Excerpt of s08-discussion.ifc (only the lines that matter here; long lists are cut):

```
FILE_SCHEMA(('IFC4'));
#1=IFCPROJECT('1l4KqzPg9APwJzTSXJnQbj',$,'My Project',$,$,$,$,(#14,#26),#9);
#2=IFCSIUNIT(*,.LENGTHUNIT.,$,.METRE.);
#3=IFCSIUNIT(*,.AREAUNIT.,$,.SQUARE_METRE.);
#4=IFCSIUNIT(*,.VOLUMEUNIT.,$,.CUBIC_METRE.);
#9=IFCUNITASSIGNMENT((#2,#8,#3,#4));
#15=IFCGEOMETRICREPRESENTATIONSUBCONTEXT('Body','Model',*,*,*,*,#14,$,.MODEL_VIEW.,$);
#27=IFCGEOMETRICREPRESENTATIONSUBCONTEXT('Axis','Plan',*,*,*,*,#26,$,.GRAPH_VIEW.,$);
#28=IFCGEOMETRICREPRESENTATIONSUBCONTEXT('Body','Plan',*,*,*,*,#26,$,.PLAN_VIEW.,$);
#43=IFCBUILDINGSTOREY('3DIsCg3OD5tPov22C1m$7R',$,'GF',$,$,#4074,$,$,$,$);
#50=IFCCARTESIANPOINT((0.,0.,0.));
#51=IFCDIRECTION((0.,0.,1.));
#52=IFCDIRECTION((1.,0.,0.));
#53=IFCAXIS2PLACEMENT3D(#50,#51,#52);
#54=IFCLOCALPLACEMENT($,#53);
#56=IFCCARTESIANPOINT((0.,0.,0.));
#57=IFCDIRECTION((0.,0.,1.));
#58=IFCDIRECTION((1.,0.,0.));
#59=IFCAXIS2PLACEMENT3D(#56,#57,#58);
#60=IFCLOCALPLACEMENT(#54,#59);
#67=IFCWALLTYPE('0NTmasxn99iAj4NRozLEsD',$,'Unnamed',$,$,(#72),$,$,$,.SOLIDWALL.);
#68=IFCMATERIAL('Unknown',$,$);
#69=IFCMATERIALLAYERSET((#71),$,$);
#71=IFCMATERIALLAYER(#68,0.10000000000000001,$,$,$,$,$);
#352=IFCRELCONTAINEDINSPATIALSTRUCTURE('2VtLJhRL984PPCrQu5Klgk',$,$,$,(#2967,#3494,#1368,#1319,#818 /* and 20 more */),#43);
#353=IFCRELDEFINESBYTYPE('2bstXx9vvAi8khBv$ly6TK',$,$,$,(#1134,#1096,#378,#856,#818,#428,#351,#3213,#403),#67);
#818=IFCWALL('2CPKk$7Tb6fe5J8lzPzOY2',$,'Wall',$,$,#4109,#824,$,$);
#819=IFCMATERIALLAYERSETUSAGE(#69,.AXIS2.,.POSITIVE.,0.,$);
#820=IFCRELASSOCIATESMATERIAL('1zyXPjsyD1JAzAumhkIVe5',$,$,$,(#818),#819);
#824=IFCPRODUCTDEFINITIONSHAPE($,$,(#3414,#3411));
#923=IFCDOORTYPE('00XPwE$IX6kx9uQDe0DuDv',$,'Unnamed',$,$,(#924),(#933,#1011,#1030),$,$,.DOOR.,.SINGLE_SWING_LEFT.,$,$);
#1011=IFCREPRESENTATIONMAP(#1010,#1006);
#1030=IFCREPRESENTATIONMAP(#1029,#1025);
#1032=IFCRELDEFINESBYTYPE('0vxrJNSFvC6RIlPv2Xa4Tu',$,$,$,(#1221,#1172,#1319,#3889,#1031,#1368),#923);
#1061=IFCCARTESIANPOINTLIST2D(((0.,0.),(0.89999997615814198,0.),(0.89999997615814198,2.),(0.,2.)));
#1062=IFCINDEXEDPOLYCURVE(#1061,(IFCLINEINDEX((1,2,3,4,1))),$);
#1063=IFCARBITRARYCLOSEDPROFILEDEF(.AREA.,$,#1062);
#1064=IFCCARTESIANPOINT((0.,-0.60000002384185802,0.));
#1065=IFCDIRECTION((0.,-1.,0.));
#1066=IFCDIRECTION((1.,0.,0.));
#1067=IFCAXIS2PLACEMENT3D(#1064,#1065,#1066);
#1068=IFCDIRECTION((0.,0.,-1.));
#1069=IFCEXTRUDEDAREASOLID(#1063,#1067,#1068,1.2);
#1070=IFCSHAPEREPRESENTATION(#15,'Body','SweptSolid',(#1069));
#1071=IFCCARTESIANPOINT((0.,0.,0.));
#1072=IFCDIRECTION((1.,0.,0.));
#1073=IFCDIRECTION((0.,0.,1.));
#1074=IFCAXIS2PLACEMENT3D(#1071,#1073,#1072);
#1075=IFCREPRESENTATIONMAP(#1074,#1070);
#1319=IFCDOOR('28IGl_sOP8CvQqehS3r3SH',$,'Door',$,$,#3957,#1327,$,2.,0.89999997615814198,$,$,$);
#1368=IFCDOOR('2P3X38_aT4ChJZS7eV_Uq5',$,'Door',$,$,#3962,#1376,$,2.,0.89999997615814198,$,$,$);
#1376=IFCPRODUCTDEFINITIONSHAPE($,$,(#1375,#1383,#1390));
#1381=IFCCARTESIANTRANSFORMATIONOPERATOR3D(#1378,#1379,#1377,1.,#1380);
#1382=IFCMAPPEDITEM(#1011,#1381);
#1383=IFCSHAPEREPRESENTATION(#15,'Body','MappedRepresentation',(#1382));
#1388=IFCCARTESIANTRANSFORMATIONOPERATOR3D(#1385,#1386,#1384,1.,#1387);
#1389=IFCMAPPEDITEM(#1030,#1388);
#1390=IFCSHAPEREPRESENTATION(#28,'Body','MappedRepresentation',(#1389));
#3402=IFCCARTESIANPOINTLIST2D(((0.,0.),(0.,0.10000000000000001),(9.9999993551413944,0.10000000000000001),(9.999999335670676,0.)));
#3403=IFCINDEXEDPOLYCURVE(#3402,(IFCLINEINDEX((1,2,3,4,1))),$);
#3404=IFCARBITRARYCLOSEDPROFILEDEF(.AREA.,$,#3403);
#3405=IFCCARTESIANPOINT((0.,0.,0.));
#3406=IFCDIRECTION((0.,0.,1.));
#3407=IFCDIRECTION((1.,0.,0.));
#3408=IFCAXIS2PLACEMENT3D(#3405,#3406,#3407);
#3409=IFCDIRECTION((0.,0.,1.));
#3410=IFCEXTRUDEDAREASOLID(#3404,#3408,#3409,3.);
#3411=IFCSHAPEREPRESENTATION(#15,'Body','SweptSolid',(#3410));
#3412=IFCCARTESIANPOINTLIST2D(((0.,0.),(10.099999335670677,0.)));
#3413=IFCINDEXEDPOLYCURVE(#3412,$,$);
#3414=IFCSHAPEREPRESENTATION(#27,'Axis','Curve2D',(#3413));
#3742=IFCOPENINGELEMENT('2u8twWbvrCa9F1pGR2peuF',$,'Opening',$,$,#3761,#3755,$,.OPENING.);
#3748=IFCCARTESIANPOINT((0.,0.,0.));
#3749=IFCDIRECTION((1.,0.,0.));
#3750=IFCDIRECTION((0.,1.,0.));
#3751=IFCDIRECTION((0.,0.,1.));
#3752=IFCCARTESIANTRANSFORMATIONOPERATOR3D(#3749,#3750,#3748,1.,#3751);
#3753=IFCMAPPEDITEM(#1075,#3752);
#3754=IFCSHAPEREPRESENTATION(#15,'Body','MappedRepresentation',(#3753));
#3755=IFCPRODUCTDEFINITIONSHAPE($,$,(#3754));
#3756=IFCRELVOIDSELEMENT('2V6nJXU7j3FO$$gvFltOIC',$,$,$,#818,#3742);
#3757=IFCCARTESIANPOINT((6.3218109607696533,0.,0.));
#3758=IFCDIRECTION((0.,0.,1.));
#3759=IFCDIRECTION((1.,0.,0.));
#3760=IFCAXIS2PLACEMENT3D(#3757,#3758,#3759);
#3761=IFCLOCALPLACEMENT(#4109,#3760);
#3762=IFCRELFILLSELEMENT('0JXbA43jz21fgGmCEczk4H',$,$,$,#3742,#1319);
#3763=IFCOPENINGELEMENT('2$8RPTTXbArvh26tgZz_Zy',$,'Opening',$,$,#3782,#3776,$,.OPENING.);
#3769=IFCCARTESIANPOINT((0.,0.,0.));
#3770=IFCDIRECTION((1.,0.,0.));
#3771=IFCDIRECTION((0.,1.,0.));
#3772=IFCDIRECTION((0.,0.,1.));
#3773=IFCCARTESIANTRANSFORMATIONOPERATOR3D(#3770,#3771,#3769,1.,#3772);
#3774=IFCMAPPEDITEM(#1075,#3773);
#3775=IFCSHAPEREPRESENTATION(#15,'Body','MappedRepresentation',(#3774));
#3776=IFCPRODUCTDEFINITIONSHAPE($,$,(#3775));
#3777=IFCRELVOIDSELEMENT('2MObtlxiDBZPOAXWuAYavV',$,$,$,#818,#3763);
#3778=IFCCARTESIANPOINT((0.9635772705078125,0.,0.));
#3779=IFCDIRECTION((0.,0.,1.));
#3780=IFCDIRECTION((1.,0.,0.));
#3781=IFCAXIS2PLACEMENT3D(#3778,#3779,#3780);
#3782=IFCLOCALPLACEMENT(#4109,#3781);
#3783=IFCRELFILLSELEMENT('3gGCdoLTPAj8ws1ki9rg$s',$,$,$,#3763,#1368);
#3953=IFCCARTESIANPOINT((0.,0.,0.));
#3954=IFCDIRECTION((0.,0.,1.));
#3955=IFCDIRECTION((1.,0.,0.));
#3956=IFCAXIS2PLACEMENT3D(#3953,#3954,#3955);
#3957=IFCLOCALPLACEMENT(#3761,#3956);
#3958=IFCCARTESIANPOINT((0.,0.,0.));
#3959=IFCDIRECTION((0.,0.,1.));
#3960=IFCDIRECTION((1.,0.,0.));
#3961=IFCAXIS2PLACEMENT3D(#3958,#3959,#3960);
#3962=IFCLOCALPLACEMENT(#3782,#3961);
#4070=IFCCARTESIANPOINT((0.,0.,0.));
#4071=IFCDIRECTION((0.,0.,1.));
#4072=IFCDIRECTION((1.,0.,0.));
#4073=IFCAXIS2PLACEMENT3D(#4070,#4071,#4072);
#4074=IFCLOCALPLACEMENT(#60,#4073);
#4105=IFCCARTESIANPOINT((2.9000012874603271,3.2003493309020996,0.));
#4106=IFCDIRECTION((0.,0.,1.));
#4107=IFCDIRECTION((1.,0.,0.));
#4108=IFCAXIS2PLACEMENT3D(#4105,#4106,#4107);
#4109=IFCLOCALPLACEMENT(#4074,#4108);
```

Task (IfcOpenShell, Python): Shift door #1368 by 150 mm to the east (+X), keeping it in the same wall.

```python
import ifcopenshell
import ifcopenshell.api.geometry
import ifcopenshell.util.placement
import ifcopenshell.util.unit

model = ifcopenshell.open("s08-discussion.ifc")
unit_scale = ifcopenshell.util.unit.calculate_unit_scale(model)

door = model.by_guid("2P3X38_aT4ChJZS7eV_Uq5")
opening = door.FillsVoids[0].RelatingOpeningElement
wall = opening.VoidsElements[0].RelatingBuildingElement

wall_matrix = ifcopenshell.util.placement.get_local_placement(wall.ObjectPlacement)
shift = wall_matrix[:3, 0] * 0.15 / unit_scale
before = ifcopenshell.util.placement.get_local_placement(door.ObjectPlacement)[:3, 3].copy()

# The door is placed relative to its opening, so it follows when the opening moves.
matrix = ifcopenshell.util.placement.get_local_placement(opening.ObjectPlacement)
matrix[:3, 3] += shift
ifcopenshell.api.geometry.edit_object_placement(
    model, product=opening, matrix=matrix, is_si=False, should_transform_children=True
)

after = ifcopenshell.util.placement.get_local_placement(door.ObjectPlacement)[:3, 3]
print("door moved by", (after - before).round(3) + 0.0)

model.write("s08-discussion-out.ifc")
```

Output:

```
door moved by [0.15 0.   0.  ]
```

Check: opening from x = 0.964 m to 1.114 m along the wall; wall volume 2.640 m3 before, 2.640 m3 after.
